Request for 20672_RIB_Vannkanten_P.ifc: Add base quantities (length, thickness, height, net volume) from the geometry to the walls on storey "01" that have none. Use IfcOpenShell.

First a look at what the model holds.

```python
import ifcopenshell
import ifcopenshell.util.element
import ifcopenshell.util.unit

model = ifcopenshell.open("20672_RIB_Vannkanten_P.ifc")
print(model.schema)
for unit_type in ("LENGTHUNIT", "AREAUNIT", "VOLUMEUNIT"):
    print(unit_type, ifcopenshell.util.unit.calculate_unit_scale(model, unit_type))
storey = next(s for s in model.by_type("IfcBuildingStorey") if s.Name == "01")
walls = [e for e in ifcopenshell.util.element.get_decomposition(storey) if e.is_a("IfcWall")]
for e in sorted(walls, key=lambda e: e.id()):
    print(e.id(), e.is_a(), e.Name, list(ifcopenshell.util.element.get_psets(e, qtos_only=True)), sep=" | ")
```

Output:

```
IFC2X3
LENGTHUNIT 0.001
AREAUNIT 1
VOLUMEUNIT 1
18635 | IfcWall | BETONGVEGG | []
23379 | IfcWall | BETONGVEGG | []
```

```python
import ifcopenshell
import ifcopenshell.api.pset
import ifcopenshell.geom
import ifcopenshell.util.element
import ifcopenshell.util.shape
import ifcopenshell.util.unit

model = ifcopenshell.open("20672_RIB_Vannkanten_P.ifc")
unit_scale = ifcopenshell.util.unit.calculate_unit_scale(model)
volume_scale = ifcopenshell.util.unit.calculate_unit_scale(model, "VOLUMEUNIT")
settings = ifcopenshell.geom.settings()

storey = next(s for s in model.by_type("IfcBuildingStorey") if s.Name == "01")
walls = [e for e in ifcopenshell.util.element.get_decomposition(storey) if e.is_a("IfcWall")]

for e in sorted(walls, key=lambda e: e.id()):
    if ifcopenshell.util.element.get_psets(e, qtos_only=True, should_inherit=False):
        continue
    # Geometry comes back in metres, in the element's own axes.
    shape = ifcopenshell.geom.create_shape(settings, e)
    values = {
        "Length": ifcopenshell.util.shape.get_x(shape.geometry) / unit_scale,
        "Width": ifcopenshell.util.shape.get_y(shape.geometry) / unit_scale,
        "Height": ifcopenshell.util.shape.get_z(shape.geometry) / unit_scale,
        "NetVolume": ifcopenshell.util.shape.get_volume(shape.geometry) / volume_scale,
    }
    qto = ifcopenshell.api.pset.add_qto(model, product=e, name="BaseQuantities")
    ifcopenshell.api.pset.edit_qto(model, qto=qto, properties=values)
    print(e.id(), {k: round(v, 3) for k, v in values.items()})

model.write("20672_RIB_Vannkanten_P_edited.ifc")
```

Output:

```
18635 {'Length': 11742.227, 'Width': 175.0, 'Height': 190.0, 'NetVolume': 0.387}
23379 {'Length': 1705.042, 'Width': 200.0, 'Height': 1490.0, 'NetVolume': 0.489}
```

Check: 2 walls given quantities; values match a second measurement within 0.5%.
